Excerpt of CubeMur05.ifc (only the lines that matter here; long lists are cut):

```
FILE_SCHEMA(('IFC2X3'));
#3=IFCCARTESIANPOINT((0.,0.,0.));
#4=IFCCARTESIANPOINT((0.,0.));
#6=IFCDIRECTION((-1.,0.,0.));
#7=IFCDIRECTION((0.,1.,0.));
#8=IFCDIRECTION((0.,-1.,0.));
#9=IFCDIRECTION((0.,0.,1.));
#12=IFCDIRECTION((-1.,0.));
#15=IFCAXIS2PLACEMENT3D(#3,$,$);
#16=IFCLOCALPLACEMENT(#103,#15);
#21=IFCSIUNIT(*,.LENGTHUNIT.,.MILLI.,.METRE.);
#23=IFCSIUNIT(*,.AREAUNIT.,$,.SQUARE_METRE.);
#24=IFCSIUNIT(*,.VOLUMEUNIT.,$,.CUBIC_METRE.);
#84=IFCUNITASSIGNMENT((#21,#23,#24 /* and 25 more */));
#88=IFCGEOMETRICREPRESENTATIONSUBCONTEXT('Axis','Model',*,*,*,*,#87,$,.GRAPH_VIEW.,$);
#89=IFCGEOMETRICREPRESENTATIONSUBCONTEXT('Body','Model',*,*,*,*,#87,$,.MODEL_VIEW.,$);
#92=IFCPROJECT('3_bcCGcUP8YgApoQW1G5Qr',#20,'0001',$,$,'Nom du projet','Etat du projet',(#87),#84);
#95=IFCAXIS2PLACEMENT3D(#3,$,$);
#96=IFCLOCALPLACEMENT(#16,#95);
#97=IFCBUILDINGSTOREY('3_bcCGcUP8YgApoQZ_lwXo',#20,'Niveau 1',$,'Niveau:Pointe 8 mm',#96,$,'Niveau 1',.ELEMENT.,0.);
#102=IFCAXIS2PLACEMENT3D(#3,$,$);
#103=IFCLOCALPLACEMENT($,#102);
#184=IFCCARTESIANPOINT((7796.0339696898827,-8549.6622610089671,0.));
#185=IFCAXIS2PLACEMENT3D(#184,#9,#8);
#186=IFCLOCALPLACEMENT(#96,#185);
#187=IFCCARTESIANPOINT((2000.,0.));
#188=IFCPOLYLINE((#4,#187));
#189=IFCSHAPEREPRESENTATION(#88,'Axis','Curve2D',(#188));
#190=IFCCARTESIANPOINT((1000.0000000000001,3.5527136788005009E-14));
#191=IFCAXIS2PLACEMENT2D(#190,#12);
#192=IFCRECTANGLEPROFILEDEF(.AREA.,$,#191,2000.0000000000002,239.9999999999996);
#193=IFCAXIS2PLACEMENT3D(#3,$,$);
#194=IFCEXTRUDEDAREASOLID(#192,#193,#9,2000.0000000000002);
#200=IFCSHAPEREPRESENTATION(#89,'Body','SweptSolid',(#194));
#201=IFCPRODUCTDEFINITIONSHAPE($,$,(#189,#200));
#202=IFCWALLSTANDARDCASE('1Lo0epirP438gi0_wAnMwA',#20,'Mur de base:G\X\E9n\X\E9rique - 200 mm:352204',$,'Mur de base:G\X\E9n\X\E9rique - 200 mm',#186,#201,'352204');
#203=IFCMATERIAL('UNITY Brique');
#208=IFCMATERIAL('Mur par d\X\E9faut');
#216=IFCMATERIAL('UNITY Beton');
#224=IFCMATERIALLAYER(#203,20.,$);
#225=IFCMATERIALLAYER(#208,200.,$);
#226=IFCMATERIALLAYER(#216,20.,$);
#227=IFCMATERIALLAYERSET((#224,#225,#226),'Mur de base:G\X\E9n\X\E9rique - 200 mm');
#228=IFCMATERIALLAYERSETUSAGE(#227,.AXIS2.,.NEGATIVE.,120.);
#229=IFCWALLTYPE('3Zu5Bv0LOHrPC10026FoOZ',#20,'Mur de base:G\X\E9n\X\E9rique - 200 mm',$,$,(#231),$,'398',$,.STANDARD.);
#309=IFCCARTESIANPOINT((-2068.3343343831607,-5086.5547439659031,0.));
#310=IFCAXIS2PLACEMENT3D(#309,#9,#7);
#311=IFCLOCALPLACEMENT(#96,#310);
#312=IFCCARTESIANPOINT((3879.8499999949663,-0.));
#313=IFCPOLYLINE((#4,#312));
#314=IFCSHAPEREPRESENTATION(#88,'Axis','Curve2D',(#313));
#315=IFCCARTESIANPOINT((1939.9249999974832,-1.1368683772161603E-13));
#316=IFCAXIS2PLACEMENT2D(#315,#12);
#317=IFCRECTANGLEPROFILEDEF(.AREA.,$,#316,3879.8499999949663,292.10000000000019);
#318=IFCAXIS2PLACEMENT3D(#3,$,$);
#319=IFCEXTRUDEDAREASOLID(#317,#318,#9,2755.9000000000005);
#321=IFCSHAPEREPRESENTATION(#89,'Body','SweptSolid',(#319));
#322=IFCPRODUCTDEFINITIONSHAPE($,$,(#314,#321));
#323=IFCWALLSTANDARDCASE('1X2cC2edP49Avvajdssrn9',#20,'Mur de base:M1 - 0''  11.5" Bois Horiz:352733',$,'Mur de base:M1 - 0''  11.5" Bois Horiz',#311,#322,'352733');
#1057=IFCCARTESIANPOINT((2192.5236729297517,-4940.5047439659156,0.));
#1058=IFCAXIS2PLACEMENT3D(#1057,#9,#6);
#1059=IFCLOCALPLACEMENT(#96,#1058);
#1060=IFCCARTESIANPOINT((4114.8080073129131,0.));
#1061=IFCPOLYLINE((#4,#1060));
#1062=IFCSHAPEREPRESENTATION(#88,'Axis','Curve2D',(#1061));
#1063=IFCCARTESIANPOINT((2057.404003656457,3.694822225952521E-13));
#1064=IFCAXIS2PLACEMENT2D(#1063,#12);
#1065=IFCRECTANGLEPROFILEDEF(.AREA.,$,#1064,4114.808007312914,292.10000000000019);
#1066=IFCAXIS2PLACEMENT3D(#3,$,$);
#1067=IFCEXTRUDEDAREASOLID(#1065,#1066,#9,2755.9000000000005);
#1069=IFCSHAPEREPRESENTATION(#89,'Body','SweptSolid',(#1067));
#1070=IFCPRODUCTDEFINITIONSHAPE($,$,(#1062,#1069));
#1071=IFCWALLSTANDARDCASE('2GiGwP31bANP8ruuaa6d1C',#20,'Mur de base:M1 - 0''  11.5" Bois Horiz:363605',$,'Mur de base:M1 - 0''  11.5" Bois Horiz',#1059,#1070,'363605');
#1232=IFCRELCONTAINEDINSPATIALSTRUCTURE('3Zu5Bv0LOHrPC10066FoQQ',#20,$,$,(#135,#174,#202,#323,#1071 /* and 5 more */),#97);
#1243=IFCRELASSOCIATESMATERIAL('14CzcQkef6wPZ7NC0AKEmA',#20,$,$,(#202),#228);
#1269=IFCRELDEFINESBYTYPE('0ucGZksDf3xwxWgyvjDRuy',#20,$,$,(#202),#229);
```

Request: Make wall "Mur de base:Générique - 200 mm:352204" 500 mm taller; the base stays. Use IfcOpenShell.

```python
import ifcopenshell
import ifcopenshell.geom
import ifcopenshell.util.representation
import ifcopenshell.util.shape
import ifcopenshell.util.unit

model = ifcopenshell.open("CubeMur05.ifc")
unit_scale = ifcopenshell.util.unit.calculate_unit_scale(model)
settings = ifcopenshell.geom.settings()


def volume(element):
    """Net volume in cubic metres, openings subtracted."""
    shape = ifcopenshell.geom.create_shape(settings, element)
    return ifcopenshell.util.shape.get_volume(shape.geometry)


wall = model.by_id(202)
before = volume(wall)

body = ifcopenshell.util.representation.get_representation(wall, "Model", "Body")
solid = body.Items[0]
old_height = solid.Depth
solid.Depth += 0.5 / unit_scale
after = volume(wall)

print(f"height {old_height:g} -> {solid.Depth:g}, volume {before:.3f} -> {after:.3f} m3")

model.write("CubeMur05-out.ifc")
```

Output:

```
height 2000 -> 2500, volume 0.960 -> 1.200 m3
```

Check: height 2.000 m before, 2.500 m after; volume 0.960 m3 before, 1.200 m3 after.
